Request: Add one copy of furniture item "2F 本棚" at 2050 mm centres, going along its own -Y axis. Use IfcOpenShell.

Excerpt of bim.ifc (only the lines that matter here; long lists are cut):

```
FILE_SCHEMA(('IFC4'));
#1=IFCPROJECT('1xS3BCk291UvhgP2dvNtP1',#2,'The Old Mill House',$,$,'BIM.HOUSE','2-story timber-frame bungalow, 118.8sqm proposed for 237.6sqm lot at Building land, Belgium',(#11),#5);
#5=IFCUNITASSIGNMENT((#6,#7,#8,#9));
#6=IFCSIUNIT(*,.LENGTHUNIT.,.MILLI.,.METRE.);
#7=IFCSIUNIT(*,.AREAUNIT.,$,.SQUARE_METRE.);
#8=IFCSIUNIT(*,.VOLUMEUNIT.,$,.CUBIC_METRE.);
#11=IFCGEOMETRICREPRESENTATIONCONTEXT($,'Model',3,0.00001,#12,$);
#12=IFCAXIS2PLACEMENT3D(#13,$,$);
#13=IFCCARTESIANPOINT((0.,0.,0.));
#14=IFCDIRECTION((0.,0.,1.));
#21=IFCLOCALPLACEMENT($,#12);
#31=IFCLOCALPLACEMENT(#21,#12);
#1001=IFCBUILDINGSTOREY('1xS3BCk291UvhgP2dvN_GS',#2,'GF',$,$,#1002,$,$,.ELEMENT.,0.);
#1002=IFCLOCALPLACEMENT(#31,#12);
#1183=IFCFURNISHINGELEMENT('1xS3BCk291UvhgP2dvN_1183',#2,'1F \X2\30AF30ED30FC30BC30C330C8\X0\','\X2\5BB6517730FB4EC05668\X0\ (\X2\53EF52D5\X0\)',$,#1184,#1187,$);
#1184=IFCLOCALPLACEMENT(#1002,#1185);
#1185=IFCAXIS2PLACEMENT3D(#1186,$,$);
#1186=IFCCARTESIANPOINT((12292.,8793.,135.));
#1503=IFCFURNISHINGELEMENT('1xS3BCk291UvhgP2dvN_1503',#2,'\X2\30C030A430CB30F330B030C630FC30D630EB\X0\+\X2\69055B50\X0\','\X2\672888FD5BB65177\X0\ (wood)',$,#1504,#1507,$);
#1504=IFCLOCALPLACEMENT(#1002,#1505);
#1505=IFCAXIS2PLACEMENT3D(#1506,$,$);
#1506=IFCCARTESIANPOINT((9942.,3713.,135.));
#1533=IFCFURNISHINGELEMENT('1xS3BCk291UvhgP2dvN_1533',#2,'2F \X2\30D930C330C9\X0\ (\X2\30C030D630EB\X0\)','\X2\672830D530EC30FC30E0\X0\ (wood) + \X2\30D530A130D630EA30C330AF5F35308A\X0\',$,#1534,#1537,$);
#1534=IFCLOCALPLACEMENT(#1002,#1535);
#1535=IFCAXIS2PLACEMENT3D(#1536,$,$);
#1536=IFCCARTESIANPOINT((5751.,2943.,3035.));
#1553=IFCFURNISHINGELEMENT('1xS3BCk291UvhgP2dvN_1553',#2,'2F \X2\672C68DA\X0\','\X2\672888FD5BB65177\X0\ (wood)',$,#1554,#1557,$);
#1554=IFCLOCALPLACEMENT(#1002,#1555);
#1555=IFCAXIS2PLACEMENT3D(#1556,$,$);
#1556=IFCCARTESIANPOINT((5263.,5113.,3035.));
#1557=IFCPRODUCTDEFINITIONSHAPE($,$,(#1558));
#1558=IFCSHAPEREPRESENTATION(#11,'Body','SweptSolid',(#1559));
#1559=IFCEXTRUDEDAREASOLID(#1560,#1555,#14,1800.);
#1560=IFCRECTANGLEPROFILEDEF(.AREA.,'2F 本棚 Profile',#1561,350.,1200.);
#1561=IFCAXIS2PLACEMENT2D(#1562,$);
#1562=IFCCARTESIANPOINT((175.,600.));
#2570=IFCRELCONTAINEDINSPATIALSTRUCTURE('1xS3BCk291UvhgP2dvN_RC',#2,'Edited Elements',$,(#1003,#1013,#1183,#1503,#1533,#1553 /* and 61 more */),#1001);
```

```python
import ifcopenshell
import ifcopenshell.api.geometry
import ifcopenshell.api.root
import ifcopenshell.util.element
import ifcopenshell.util.placement
import ifcopenshell.util.unit

model = ifcopenshell.open("bim.ifc")
unit_scale = ifcopenshell.util.unit.calculate_unit_scale(model)


def reuse_history(source, copy):
    """copy_class also copies each property set's owner history, people and application; keep the originals."""
    for rel in copy.IsDefinedBy:
        if rel.is_a("IfcRelDefinesByProperties") and (history := rel.RelatingPropertyDefinition.OwnerHistory):
            rel.RelatingPropertyDefinition.OwnerHistory = source.OwnerHistory
            ifcopenshell.util.element.remove_deep2(model, history)


source = model.by_guid("1xS3BCk291UvhgP2dvN_1553")
base = ifcopenshell.util.placement.get_local_placement(source.ObjectPlacement)
step = -base[:3, 1] * 2.05 / unit_scale

for i in range(1, 2):
    copy = ifcopenshell.api.root.copy_class(model, product=source)
    copy.Representation = ifcopenshell.util.element.copy_deep(
        model, source.Representation, exclude=["IfcGeometricRepresentationContext", "IfcRepresentationMap"]
    )
    reuse_history(source, copy)
    matrix = base.copy()
    matrix[:3, 3] += i * step
    print("added at", matrix[:3, 3].round(3) + 0.0)
    ifcopenshell.api.geometry.edit_object_placement(model, product=copy, matrix=matrix, is_si=False)

model.write("bim_updated.ifc")
```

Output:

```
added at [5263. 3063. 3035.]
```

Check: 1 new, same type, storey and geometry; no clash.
